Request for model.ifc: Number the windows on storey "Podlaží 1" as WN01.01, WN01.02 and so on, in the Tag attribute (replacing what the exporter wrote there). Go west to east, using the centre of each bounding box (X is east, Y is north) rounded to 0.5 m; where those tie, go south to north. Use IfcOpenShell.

First a look at what the model holds.

```python
import ifcopenshell
import ifcopenshell.util.element
import ifcopenshell.util.placement

model = ifcopenshell.open("model.ifc")
print(model.schema)
storey = next(s for s in model.by_type("IfcBuildingStorey") if s.Name == "Podlaží 1")
windows = [e for e in ifcopenshell.util.element.get_decomposition(storey) if e.is_a("IfcWindow")]
for e in sorted(windows, key=lambda e: e.id()):
    origin = ifcopenshell.util.placement.get_local_placement(e.ObjectPlacement)[:3, 3]
    print(e.id(), e.Tag, e.Name, origin.round(2) + 0.0, sep=" | ")
```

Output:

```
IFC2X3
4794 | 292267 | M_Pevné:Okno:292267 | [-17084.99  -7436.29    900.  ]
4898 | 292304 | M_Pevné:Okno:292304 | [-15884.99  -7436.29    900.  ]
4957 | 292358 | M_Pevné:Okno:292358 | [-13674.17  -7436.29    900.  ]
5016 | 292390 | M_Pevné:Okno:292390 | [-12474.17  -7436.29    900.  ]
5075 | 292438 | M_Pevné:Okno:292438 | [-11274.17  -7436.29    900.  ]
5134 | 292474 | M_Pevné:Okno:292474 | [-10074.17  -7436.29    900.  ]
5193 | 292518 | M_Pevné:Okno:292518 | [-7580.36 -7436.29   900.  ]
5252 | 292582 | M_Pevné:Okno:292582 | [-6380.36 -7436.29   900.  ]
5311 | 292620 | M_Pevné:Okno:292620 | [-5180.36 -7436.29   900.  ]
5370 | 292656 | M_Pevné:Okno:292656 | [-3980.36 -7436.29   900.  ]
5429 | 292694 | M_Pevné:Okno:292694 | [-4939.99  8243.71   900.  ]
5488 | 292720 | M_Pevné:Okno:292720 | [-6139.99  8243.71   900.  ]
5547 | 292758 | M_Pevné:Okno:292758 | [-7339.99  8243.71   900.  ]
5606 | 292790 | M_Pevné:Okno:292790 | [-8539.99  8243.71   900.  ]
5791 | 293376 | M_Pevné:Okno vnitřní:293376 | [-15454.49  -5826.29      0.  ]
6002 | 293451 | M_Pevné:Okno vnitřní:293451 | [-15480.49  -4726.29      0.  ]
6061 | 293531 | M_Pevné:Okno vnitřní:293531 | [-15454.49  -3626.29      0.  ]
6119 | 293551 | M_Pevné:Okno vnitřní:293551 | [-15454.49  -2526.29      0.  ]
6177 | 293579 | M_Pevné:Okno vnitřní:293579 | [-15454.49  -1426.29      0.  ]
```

```python
import ifcopenshell
import ifcopenshell.geom
import ifcopenshell.util.element
import ifcopenshell.util.shape

model = ifcopenshell.open("model.ifc")
settings = ifcopenshell.geom.settings()
settings.set("use-world-coords", True)


def centre(element):
    shape = ifcopenshell.geom.create_shape(settings, element)
    return ifcopenshell.util.shape.get_bbox_centroid(shape.geometry)


storey = next(s for s in model.by_type("IfcBuildingStorey") if s.Name == "Podlaží 1")
windows = [e for e in ifcopenshell.util.element.get_decomposition(storey) if e.is_a("IfcWindow")]

# Insertion points can sit at a corner or the storey origin, so sort by the geometry (in metres).
centres = {e: centre(e) for e in windows}
windows.sort(key=lambda e: (round(centres[e][0] / 0.5), centres[e][1]))

for i, e in enumerate(windows, start=1):
    number = f"WN01.{i:02d}"
    e.Tag = number
    print(e.id(), number)

model.write("model_edited.ifc")
```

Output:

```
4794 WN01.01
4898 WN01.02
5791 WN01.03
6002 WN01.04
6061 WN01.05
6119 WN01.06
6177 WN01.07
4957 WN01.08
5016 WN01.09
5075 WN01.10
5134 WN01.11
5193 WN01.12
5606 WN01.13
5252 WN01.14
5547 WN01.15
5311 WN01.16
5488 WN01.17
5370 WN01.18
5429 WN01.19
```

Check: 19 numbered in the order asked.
